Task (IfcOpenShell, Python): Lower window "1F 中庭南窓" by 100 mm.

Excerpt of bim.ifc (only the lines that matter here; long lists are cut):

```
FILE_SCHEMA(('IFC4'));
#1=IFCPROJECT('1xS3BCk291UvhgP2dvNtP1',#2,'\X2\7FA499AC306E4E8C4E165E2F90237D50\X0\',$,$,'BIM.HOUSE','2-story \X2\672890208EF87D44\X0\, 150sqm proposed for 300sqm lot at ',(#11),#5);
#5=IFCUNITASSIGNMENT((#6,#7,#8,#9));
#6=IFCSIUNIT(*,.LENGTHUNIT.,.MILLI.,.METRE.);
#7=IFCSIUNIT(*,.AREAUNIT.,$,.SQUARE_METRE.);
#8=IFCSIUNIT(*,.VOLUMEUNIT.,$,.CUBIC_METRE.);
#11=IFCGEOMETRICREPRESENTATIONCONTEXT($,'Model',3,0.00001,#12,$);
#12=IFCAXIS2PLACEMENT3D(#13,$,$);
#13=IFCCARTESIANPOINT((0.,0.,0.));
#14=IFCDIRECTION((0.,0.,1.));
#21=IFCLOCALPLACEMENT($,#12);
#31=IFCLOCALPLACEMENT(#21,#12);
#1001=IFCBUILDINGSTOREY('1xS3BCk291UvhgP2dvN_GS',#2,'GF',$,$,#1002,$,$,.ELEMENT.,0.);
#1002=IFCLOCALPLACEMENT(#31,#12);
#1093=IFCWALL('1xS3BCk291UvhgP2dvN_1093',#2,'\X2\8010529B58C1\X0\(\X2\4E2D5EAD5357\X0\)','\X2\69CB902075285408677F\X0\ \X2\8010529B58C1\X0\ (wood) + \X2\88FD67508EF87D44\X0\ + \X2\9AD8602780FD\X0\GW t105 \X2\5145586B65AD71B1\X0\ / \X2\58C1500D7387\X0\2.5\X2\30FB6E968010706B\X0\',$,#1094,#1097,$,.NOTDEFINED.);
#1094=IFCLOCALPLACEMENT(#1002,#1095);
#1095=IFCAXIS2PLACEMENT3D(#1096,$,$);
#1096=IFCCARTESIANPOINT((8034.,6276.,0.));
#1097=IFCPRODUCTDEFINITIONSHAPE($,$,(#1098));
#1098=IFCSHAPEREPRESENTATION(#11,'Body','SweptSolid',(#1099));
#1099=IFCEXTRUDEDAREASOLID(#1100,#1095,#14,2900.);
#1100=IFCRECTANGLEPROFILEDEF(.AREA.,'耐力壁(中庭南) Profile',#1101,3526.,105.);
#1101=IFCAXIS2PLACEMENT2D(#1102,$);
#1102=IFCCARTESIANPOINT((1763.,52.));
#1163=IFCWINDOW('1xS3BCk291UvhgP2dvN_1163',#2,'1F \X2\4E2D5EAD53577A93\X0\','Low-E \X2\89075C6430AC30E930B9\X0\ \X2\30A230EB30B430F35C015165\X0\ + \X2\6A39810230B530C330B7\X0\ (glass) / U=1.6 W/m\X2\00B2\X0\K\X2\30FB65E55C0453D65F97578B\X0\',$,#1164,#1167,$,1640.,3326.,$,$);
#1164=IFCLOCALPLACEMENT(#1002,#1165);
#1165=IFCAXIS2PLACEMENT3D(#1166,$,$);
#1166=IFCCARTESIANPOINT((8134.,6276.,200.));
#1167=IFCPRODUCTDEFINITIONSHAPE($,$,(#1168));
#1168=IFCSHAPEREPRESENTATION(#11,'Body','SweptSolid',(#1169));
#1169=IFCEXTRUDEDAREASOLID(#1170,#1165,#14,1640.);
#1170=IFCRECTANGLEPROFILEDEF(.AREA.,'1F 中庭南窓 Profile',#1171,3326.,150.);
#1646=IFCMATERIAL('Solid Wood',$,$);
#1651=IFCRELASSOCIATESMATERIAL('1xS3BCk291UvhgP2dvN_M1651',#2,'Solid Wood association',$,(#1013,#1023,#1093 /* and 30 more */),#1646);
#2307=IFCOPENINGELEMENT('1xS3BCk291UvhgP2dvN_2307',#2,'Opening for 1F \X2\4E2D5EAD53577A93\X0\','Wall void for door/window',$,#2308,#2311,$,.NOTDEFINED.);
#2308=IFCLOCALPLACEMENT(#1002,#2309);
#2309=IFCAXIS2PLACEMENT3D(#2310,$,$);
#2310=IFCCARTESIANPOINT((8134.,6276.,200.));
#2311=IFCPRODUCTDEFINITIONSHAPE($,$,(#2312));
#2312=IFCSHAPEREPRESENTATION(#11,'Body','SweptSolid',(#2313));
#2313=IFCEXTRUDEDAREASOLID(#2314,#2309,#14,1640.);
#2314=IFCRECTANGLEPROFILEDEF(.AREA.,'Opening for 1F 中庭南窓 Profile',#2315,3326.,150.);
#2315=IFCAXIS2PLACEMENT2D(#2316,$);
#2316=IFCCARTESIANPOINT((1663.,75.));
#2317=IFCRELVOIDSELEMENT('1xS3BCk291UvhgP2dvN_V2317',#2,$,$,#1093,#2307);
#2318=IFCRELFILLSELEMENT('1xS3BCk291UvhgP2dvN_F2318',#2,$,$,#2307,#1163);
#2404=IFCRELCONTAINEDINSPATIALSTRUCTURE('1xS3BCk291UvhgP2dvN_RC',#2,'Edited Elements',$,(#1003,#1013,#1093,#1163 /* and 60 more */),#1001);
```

```python
import numpy as np
import ifcopenshell
import ifcopenshell.api.geometry
import ifcopenshell.util.placement
import ifcopenshell.util.unit

model = ifcopenshell.open("bim.ifc")
unit_scale = ifcopenshell.util.unit.calculate_unit_scale(model)

window = model.by_guid("1xS3BCk291UvhgP2dvN_1163")
opening = window.FillsVoids[0].RelatingOpeningElement
dz = -0.1 / unit_scale

shift = np.array([0.0, 0.0, dz])
# The window is not placed relative to its opening, so move both.
for product in (opening, window):
    matrix = ifcopenshell.util.placement.get_local_placement(product.ObjectPlacement)
    matrix[:3, 3] += shift
    ifcopenshell.api.geometry.edit_object_placement(model, product=product, matrix=matrix, is_si=False)

print(f"moved by {dz * unit_scale:+.3f} m")

model.write("bim-out.ifc")
```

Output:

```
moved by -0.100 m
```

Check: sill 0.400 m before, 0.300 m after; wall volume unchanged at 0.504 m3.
